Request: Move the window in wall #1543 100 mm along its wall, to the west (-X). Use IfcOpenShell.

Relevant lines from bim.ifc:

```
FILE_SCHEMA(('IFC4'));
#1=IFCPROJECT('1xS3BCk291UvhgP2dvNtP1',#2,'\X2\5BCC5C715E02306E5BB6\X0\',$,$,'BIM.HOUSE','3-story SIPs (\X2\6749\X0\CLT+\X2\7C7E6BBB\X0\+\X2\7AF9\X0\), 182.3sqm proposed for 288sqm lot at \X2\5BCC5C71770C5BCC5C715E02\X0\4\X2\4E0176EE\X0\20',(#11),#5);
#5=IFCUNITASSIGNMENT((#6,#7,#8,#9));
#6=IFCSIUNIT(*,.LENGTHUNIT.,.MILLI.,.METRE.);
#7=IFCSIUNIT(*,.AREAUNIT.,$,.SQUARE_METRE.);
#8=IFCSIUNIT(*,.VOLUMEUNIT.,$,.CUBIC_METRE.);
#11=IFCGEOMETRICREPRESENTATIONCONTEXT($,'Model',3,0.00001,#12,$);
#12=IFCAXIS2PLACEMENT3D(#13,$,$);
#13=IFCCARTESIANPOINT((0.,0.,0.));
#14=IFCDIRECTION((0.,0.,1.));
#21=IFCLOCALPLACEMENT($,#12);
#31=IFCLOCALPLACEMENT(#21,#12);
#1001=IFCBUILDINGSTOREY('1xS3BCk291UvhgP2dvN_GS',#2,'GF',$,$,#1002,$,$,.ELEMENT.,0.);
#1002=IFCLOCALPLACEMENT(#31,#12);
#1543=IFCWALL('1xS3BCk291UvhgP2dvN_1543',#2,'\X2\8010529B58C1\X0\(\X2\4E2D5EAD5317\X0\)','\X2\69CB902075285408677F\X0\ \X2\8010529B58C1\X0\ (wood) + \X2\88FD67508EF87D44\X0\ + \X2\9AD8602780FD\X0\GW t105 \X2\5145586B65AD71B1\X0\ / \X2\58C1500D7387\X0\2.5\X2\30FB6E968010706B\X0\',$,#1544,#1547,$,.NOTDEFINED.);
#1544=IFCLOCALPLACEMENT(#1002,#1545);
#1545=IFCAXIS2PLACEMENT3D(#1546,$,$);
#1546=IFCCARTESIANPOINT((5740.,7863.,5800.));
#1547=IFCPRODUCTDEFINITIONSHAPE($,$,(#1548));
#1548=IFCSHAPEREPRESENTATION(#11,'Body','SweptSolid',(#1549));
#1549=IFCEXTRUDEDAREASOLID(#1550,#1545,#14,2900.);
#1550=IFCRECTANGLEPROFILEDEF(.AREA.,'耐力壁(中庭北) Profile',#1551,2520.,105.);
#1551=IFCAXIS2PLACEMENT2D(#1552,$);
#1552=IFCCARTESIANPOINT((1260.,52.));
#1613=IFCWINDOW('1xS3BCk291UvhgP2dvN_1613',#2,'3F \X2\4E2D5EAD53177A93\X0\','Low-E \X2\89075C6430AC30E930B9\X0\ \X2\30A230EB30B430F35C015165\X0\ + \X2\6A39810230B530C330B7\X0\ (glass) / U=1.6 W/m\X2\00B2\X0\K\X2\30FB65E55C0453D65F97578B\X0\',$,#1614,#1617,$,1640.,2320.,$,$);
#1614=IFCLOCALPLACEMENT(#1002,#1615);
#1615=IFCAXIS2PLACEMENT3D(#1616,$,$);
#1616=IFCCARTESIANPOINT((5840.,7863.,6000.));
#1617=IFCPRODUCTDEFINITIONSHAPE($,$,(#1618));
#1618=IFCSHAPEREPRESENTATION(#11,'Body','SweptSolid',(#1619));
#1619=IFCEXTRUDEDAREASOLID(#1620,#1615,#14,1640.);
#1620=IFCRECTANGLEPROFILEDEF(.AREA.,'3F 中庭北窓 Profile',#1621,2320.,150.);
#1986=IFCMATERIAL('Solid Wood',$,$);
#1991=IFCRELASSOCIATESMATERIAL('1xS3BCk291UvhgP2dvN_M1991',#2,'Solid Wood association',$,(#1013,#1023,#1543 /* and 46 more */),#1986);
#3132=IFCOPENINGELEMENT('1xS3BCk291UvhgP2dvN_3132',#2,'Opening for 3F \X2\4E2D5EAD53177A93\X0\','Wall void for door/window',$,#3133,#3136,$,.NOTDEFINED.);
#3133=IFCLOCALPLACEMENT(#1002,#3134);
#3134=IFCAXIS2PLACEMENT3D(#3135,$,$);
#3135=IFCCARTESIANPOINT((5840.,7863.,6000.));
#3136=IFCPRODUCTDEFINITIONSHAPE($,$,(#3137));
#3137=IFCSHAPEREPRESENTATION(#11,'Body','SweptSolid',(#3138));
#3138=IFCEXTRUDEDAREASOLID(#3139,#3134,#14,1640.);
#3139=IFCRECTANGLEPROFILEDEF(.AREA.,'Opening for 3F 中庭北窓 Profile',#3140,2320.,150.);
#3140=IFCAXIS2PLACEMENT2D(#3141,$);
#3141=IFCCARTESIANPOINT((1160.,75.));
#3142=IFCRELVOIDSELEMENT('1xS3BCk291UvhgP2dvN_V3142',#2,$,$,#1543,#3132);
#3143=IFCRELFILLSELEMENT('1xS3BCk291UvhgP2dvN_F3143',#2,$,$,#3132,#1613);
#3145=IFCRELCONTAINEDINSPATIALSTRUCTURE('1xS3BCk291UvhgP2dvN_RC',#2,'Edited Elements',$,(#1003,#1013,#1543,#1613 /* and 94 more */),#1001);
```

```python
import ifcopenshell
import ifcopenshell.api.geometry
import ifcopenshell.util.placement
import ifcopenshell.util.unit

model = ifcopenshell.open("bim.ifc")
unit_scale = ifcopenshell.util.unit.calculate_unit_scale(model)

window = model.by_guid("1xS3BCk291UvhgP2dvN_1613")
opening = window.FillsVoids[0].RelatingOpeningElement
wall = opening.VoidsElements[0].RelatingBuildingElement

wall_matrix = ifcopenshell.util.placement.get_local_placement(wall.ObjectPlacement)
shift = wall_matrix[:3, 0] * -0.1 / unit_scale
before = ifcopenshell.util.placement.get_local_placement(window.ObjectPlacement)[:3, 3].copy()

# The window is not placed relative to its opening, so move both.
for product in (opening, window):
    matrix = ifcopenshell.util.placement.get_local_placement(product.ObjectPlacement)
    matrix[:3, 3] += shift
    ifcopenshell.api.geometry.edit_object_placement(model, product=product, matrix=matrix, is_si=False)

after = ifcopenshell.util.placement.get_local_placement(window.ObjectPlacement)[:3, 3]
print("window moved by", (after - before).round(3) + 0.0)

model.write("bim_v2.ifc")
```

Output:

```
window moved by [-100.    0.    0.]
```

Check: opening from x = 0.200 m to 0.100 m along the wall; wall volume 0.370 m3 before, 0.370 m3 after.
